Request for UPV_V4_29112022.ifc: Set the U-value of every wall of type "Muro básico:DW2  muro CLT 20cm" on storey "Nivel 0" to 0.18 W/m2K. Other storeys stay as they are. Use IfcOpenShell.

First a look at what the model holds.

```python
import ifcopenshell
import ifcopenshell.util.element

model = ifcopenshell.open("UPV_V4_29112022.ifc")
print(model.schema)
storey = next(s for s in model.by_type("IfcBuildingStorey") if s.Name == "Nivel 0")
walls = [e for e in ifcopenshell.util.element.get_decomposition(storey) if e.is_a("IfcWall")]
seen = {}
for e in walls:
    element_type = ifcopenshell.util.element.get_type(e)
    key = (element_type.Name if element_type != e and element_type else None, ifcopenshell.util.element.get_pset(e, "Pset_WallCommon", "ThermalTransmittance"))
    seen[key] = seen.get(key, 0) + 1
for (name, value), count in sorted(seen.items(), key=str):
    print(count, "x", name, "|", value)
```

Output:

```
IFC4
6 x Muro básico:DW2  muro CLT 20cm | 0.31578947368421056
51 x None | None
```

```python
import ifcopenshell
import ifcopenshell.api.pset
import ifcopenshell.util.element

model = ifcopenshell.open("UPV_V4_29112022.ifc")

storey = next(s for s in model.by_type("IfcBuildingStorey") if s.Name == "Nivel 0")
walls = [e for e in ifcopenshell.util.element.get_decomposition(storey) if e.is_a("IfcWall")]

count = 0
for e in walls:
    element_type = ifcopenshell.util.element.get_type(e)
    if element_type in (None, e) or element_type.Name != "Muro básico:DW2  muro CLT 20cm":
        continue
    # add_pset returns the element's existing set when there is one.
    pset = ifcopenshell.api.pset.add_pset(model, product=e, name="Pset_WallCommon")
    ifcopenshell.api.pset.edit_pset(model, pset=pset, properties={"ThermalTransmittance": 0.18})
    count += 1

print(count, "walls updated")

model.write("UPV_V4_29112022_rev.ifc")
```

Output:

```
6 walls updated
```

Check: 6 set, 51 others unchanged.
